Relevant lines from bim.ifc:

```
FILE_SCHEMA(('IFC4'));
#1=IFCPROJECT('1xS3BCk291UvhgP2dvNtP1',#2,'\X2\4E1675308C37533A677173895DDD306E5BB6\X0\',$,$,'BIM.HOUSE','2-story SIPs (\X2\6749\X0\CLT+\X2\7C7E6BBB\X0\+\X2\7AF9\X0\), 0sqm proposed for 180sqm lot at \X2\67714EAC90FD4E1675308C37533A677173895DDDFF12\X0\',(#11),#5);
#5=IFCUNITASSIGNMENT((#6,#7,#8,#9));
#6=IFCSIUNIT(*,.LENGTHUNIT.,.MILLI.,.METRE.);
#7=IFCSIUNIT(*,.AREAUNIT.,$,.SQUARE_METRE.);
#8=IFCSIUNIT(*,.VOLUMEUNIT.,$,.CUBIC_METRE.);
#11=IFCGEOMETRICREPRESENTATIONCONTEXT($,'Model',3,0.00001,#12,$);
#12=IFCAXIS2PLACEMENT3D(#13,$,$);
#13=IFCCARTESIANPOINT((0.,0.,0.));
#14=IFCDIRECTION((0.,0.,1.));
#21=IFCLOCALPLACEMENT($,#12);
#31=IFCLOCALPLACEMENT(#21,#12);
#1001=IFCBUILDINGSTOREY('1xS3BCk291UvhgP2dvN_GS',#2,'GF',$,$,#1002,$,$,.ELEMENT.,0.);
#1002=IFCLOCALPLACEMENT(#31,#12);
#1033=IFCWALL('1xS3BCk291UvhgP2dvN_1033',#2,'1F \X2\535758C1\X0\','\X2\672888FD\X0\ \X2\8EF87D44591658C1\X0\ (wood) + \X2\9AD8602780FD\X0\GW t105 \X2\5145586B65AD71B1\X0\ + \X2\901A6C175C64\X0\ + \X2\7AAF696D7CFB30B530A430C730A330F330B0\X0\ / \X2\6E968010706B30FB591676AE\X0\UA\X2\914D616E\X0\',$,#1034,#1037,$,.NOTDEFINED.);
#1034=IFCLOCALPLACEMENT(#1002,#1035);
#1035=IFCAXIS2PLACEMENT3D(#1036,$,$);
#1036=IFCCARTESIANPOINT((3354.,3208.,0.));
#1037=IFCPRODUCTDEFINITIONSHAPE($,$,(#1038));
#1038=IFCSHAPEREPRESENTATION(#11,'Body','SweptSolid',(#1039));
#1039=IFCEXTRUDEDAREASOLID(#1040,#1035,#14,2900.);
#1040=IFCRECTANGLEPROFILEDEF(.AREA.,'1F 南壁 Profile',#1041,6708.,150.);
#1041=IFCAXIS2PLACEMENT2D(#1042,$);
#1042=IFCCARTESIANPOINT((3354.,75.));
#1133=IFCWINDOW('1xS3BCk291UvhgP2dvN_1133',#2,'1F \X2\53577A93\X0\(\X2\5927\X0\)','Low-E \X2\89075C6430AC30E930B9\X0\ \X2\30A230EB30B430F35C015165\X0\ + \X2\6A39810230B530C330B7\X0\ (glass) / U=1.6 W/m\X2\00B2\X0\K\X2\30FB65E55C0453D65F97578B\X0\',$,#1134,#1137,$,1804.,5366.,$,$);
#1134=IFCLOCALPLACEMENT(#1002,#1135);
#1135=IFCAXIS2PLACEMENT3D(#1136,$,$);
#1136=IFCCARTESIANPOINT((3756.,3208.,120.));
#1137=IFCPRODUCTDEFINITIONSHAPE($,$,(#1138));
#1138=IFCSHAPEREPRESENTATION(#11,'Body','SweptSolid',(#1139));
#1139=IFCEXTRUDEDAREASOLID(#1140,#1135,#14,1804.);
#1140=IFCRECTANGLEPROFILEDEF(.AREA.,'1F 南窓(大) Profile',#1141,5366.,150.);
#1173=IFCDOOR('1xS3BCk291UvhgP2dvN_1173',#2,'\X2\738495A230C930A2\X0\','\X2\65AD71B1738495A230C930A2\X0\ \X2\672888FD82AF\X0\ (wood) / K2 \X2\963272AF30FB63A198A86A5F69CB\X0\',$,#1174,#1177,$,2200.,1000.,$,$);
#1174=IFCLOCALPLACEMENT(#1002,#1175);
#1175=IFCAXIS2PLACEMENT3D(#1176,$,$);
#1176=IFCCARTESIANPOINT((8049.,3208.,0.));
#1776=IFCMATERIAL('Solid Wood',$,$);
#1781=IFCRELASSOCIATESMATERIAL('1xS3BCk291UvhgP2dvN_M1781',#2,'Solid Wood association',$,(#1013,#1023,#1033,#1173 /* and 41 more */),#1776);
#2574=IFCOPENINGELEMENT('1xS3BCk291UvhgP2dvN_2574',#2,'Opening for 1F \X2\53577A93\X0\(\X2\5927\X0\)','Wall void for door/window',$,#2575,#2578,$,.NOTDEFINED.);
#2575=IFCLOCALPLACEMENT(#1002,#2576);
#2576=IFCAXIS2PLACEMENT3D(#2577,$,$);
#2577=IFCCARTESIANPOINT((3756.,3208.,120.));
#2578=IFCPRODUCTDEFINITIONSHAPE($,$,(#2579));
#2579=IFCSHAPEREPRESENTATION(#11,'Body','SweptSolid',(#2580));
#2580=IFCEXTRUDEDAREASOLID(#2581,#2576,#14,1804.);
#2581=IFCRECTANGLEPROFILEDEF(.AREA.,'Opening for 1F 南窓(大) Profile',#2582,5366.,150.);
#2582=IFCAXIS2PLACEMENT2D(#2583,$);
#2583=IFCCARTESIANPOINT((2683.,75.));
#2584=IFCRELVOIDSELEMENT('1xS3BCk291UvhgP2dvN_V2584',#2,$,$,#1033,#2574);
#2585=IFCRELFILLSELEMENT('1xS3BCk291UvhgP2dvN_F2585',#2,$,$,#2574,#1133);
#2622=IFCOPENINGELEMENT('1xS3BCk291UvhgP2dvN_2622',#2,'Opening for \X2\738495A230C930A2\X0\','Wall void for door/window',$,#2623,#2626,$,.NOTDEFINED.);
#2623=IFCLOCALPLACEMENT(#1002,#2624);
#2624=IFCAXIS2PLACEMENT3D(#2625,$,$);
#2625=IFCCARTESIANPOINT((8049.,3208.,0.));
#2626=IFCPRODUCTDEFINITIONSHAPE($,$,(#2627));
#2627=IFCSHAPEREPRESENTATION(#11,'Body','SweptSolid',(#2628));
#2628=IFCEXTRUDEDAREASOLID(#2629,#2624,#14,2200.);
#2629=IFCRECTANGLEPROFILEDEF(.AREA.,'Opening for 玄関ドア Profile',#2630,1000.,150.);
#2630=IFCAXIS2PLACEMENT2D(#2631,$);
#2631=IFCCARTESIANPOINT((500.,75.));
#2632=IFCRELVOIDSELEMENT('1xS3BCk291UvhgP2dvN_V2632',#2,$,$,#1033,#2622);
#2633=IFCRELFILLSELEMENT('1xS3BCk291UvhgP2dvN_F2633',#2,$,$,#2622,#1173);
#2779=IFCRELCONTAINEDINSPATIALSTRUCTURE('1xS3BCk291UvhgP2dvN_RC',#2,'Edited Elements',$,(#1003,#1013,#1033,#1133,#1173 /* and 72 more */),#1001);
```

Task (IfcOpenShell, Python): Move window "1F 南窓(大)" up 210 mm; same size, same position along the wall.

```python
import numpy as np
import ifcopenshell
import ifcopenshell.api.geometry
import ifcopenshell.util.placement
import ifcopenshell.util.unit

model = ifcopenshell.open("bim.ifc")
unit_scale = ifcopenshell.util.unit.calculate_unit_scale(model)

window = model.by_guid("1xS3BCk291UvhgP2dvN_1133")
opening = window.FillsVoids[0].RelatingOpeningElement
dz = 0.21 / unit_scale

shift = np.array([0.0, 0.0, dz])
# The window is not placed relative to its opening, so move both.
for product in (opening, window):
    matrix = ifcopenshell.util.placement.get_local_placement(product.ObjectPlacement)
    matrix[:3, 3] += shift
    ifcopenshell.api.geometry.edit_object_placement(model, product=product, matrix=matrix, is_si=False)

print(f"moved by {dz * unit_scale:+.3f} m")

model.write("bim_rev.ifc")
```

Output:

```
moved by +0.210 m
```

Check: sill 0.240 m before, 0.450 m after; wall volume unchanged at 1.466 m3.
